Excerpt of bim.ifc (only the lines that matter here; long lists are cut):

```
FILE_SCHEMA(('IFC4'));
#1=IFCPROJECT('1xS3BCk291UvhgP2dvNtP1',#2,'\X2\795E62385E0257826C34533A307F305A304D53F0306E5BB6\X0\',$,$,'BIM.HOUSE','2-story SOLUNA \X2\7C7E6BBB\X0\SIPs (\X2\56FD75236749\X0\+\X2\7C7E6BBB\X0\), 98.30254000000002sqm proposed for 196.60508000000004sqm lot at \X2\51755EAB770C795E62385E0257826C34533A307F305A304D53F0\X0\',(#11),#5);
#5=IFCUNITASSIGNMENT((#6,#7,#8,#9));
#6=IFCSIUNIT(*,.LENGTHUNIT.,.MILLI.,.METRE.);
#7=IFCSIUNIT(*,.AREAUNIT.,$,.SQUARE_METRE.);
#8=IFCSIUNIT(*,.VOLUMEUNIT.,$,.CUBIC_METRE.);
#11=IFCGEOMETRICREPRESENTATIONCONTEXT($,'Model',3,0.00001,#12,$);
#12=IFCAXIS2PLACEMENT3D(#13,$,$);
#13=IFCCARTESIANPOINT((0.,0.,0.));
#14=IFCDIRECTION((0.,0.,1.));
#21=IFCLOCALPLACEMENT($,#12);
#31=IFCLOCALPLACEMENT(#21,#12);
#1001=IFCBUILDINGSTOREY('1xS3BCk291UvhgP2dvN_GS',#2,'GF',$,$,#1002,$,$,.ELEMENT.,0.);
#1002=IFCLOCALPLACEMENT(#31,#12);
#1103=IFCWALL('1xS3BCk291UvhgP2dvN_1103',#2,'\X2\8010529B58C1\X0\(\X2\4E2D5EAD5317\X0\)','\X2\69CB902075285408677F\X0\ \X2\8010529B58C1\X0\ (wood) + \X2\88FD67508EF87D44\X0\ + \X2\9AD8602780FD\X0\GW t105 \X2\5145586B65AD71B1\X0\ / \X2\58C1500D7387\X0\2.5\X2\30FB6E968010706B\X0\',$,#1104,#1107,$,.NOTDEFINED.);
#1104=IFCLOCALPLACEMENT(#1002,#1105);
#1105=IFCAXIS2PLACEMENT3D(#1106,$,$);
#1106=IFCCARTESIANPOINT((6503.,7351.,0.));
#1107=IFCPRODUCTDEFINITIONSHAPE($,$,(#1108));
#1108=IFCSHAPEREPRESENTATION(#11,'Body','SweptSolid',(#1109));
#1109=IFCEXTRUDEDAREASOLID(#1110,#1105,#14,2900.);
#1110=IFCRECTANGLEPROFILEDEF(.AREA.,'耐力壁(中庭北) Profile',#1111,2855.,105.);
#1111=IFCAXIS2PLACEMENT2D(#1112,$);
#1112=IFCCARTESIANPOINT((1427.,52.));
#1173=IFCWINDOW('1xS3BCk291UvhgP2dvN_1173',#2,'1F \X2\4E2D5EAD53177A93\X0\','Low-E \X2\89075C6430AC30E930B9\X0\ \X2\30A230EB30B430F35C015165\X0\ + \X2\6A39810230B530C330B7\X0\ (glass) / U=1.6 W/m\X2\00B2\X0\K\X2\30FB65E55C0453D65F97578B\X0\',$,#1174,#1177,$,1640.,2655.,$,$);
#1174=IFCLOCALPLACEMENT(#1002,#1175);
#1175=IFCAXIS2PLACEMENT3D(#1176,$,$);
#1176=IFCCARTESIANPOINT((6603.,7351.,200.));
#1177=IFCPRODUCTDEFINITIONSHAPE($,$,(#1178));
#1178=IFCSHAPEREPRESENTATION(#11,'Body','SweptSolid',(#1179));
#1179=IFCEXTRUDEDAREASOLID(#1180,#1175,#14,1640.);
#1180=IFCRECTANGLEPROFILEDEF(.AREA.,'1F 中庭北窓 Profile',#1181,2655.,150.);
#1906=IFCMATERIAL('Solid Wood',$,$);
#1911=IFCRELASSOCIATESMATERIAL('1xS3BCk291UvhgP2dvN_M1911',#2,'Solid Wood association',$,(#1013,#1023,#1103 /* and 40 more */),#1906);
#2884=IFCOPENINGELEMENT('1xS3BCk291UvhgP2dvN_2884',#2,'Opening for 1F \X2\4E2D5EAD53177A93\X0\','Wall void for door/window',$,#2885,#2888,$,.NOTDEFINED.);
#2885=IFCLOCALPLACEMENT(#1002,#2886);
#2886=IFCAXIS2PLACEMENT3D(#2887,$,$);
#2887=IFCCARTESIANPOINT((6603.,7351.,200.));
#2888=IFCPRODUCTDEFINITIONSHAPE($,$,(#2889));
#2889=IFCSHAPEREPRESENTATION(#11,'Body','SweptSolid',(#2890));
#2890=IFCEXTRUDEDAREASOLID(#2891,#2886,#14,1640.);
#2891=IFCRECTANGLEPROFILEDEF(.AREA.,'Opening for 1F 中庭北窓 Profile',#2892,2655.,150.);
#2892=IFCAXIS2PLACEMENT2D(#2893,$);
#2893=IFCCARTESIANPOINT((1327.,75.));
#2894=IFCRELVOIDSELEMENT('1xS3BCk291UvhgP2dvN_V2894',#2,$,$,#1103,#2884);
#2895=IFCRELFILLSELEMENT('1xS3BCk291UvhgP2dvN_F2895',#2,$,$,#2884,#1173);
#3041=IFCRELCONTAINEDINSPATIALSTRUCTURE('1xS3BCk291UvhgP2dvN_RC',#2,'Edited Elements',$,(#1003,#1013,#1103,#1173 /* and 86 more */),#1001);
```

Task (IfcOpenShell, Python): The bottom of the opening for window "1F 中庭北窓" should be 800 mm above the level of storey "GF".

```python
import numpy as np
import ifcopenshell
import ifcopenshell.api.geometry
import ifcopenshell.geom
import ifcopenshell.util.element
import ifcopenshell.util.placement
import ifcopenshell.util.shape
import ifcopenshell.util.unit

model = ifcopenshell.open("bim.ifc")
unit_scale = ifcopenshell.util.unit.calculate_unit_scale(model)

window = model.by_guid("1xS3BCk291UvhgP2dvN_1173")
opening = window.FillsVoids[0].RelatingOpeningElement
storey = ifcopenshell.util.element.get_container(window, ifc_class="IfcBuildingStorey")
level = ifcopenshell.util.placement.get_local_placement(storey.ObjectPlacement)[2, 3]

# The opening's origin need not be at the sill, so measure its lowest point.
shape = ifcopenshell.geom.create_shape(ifcopenshell.geom.settings(), opening)
bottom = ifcopenshell.util.shape.get_shape_bottom_elevation(shape, shape.geometry) / unit_scale
dz = level + 0.8 / unit_scale - bottom

shift = np.array([0.0, 0.0, dz])
# The window is not placed relative to its opening, so move both.
for product in (opening, window):
    matrix = ifcopenshell.util.placement.get_local_placement(product.ObjectPlacement)
    matrix[:3, 3] += shift
    ifcopenshell.api.geometry.edit_object_placement(model, product=product, matrix=matrix, is_si=False)

print(f"moved by {dz * unit_scale:+.3f} m")

model.write("bim_v2.ifc")
```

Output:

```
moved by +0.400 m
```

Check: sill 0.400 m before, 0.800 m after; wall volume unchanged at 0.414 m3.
